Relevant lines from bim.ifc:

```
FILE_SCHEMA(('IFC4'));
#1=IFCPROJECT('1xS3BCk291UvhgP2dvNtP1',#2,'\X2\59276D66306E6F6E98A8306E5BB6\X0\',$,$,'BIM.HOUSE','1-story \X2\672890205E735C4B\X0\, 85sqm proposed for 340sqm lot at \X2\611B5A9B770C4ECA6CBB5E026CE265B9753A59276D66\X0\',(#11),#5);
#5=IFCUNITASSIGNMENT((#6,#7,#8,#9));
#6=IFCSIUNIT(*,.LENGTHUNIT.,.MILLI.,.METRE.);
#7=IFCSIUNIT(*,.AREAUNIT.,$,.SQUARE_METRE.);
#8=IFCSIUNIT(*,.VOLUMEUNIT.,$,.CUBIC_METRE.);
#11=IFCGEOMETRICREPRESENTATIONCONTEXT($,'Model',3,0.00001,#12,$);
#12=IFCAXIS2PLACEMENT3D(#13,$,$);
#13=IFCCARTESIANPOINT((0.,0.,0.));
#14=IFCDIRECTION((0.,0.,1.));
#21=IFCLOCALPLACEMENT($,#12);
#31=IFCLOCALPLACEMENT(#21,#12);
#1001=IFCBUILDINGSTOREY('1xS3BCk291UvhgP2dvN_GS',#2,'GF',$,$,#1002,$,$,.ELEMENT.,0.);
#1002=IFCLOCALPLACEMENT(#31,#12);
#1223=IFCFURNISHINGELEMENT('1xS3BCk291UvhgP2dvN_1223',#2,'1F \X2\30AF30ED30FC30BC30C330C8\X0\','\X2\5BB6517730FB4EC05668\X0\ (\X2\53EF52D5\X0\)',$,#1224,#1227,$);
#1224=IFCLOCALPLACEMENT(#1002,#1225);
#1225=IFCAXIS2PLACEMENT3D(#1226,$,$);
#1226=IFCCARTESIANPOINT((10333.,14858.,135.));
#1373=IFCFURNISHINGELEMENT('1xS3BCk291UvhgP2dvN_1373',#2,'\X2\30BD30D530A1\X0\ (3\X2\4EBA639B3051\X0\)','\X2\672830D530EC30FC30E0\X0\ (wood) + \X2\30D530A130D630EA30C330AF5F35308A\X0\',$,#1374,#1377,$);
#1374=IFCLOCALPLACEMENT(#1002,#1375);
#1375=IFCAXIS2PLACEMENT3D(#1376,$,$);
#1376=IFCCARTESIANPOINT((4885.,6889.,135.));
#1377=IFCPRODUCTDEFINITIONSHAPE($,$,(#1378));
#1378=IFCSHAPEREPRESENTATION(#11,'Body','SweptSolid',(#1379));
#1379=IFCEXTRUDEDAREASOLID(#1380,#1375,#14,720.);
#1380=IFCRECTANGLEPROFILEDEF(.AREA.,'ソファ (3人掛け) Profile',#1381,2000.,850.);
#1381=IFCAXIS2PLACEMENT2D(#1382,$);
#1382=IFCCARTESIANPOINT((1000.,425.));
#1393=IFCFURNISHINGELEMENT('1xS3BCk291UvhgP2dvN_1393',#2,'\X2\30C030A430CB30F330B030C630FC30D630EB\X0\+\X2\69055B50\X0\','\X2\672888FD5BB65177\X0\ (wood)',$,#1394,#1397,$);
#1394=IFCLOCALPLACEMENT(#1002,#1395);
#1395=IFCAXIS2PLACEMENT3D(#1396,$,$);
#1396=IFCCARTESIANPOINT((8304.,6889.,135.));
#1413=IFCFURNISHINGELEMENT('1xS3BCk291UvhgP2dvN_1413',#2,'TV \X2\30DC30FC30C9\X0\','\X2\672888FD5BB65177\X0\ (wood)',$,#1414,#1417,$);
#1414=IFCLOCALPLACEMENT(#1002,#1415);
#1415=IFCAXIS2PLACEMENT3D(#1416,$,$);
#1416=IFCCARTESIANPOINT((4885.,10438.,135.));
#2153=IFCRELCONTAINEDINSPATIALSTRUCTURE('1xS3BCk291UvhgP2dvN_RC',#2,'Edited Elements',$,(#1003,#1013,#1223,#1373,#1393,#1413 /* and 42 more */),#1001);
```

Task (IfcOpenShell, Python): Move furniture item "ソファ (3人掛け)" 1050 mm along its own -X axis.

```python
import ifcopenshell
import ifcopenshell.api.geometry
import ifcopenshell.util.placement

model = ifcopenshell.open("bim.ifc")

item = model.by_guid("1xS3BCk291UvhgP2dvN_1373")
matrix = ifcopenshell.util.placement.get_local_placement(item.ObjectPlacement)
matrix[:3, 3] -= matrix[:3, 0] * 1050.0
ifcopenshell.api.geometry.edit_object_placement(model, product=item, matrix=matrix, is_si=False)

print(ifcopenshell.util.placement.get_local_placement(item.ObjectPlacement).round(3) + 0.0)

model.write("bim_rev.ifc")
```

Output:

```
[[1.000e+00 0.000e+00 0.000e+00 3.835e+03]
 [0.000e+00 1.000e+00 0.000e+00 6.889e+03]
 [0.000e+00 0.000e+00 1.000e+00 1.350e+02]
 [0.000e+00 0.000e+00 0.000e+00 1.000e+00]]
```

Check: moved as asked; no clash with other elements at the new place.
